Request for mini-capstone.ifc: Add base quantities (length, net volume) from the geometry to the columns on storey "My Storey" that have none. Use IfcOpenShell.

First a look at what the model holds.

```python
import ifcopenshell
import ifcopenshell.util.element
import ifcopenshell.util.unit

model = ifcopenshell.open("mini-capstone.ifc")
print(model.schema)
for unit_type in ("LENGTHUNIT", "AREAUNIT", "VOLUMEUNIT"):
    print(unit_type, ifcopenshell.util.unit.calculate_unit_scale(model, unit_type))
storey = next(s for s in model.by_type("IfcBuildingStorey") if s.Name == "My Storey")
columns = [e for e in ifcopenshell.util.element.get_decomposition(storey) if e.is_a("IfcColumn")]
for e in sorted(columns, key=lambda e: e.id()):
    print(e.id(), e.is_a(), e.Name, list(ifcopenshell.util.element.get_psets(e, qtos_only=True)), sep=" | ")
```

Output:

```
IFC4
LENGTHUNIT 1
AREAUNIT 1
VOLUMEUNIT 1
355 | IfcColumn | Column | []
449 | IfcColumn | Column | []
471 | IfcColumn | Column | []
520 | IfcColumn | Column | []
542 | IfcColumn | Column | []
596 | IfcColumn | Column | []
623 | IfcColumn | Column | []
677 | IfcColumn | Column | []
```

```python
import ifcopenshell
import ifcopenshell.api.pset
import ifcopenshell.geom
import ifcopenshell.util.element
import ifcopenshell.util.shape
import ifcopenshell.util.unit

model = ifcopenshell.open("mini-capstone.ifc")
unit_scale = ifcopenshell.util.unit.calculate_unit_scale(model)
volume_scale = ifcopenshell.util.unit.calculate_unit_scale(model, "VOLUMEUNIT")
settings = ifcopenshell.geom.settings()

storey = next(s for s in model.by_type("IfcBuildingStorey") if s.Name == "My Storey")
columns = [e for e in ifcopenshell.util.element.get_decomposition(storey) if e.is_a("IfcColumn")]

for e in sorted(columns, key=lambda e: e.id()):
    if ifcopenshell.util.element.get_psets(e, qtos_only=True, should_inherit=False):
        continue
    # Geometry comes back in metres, in the element's own axes.
    shape = ifcopenshell.geom.create_shape(settings, e)
    values = {
        "Length": ifcopenshell.util.shape.get_z(shape.geometry) / unit_scale,
        "NetVolume": ifcopenshell.util.shape.get_volume(shape.geometry) / volume_scale,
    }
    qto = ifcopenshell.api.pset.add_qto(model, product=e, name="Qto_ColumnBaseQuantities")
    ifcopenshell.api.pset.edit_qto(model, qto=qto, properties=values)
    print(e.id(), {k: round(v, 3) for k, v in values.items()})

model.write("mini-capstone_edited.ifc")
```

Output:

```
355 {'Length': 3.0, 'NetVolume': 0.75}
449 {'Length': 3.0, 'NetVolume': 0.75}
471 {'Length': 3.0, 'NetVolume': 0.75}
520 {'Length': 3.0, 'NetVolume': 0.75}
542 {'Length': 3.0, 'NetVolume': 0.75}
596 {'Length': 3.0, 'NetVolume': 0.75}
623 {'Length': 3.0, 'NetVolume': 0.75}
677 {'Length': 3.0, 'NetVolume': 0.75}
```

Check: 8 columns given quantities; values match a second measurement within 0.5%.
